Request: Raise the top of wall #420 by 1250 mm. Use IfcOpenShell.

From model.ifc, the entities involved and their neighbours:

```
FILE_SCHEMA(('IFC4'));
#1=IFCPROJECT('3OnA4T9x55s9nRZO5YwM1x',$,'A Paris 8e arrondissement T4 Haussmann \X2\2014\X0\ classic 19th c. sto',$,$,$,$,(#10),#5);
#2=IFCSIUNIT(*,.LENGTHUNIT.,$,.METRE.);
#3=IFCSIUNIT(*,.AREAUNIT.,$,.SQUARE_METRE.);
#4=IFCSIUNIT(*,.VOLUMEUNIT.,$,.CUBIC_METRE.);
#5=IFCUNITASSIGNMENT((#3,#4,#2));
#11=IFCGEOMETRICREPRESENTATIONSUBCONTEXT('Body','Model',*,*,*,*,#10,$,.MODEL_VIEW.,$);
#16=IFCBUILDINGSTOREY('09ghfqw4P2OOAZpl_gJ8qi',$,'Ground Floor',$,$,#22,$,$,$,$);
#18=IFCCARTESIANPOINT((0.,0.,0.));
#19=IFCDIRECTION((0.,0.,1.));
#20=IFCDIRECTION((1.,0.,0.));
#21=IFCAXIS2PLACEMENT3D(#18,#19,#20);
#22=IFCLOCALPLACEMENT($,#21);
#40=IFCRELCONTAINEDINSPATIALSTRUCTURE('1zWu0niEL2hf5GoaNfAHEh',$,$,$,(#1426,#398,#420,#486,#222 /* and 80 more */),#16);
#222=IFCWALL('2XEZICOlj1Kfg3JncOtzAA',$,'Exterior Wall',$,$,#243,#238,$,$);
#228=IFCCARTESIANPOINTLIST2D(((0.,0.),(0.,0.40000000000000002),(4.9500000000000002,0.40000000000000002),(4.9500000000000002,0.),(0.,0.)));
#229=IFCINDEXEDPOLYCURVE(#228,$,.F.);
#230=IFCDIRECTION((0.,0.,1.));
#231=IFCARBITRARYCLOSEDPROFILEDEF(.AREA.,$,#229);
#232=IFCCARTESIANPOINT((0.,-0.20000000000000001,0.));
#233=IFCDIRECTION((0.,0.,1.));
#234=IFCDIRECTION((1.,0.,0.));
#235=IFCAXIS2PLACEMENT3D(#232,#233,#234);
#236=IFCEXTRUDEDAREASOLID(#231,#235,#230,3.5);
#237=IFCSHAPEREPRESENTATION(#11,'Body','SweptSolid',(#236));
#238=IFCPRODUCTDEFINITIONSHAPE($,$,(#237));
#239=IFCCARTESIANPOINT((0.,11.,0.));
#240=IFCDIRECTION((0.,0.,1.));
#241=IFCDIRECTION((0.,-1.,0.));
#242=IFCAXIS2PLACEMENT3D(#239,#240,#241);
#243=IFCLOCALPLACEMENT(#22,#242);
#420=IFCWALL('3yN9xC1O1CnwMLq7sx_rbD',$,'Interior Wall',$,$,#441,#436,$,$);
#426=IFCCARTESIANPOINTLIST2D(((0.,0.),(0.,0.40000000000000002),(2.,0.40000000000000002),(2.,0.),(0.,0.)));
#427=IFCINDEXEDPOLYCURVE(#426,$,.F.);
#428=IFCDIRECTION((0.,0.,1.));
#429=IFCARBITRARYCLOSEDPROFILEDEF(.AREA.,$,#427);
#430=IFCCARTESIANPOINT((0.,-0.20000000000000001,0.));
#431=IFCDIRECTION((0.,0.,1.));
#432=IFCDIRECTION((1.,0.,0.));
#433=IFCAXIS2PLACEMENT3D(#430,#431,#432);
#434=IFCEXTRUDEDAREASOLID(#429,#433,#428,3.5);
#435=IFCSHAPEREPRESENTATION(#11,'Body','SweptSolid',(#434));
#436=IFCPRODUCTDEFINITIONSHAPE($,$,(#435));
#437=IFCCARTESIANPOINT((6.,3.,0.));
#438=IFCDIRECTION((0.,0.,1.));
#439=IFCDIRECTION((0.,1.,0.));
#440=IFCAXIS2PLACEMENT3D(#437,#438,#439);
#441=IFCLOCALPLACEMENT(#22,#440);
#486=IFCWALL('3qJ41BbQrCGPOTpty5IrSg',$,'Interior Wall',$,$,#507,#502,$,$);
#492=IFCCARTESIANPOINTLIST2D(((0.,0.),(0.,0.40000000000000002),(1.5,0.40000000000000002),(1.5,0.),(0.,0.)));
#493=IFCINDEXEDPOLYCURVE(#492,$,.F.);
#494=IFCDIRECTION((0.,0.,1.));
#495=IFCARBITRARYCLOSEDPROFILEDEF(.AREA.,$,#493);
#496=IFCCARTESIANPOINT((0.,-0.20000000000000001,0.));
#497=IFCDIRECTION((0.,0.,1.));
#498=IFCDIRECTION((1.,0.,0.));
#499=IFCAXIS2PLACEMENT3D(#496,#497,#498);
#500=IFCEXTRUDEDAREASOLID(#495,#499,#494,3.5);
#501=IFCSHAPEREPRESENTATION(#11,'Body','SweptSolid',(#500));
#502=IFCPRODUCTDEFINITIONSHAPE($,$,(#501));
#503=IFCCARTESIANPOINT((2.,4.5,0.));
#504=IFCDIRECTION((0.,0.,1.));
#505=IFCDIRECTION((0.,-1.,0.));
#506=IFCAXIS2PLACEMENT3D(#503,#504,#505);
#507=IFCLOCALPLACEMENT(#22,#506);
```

```python
import ifcopenshell
import ifcopenshell.geom
import ifcopenshell.util.representation
import ifcopenshell.util.shape

model = ifcopenshell.open("model.ifc")
settings = ifcopenshell.geom.settings()


def volume(element):
    """Net volume in cubic metres, openings subtracted."""
    shape = ifcopenshell.geom.create_shape(settings, element)
    return ifcopenshell.util.shape.get_volume(shape.geometry)


wall = model.by_id(420)
before = volume(wall)

body = ifcopenshell.util.representation.get_representation(wall, "Model", "Body")
solid = body.Items[0]
old_height = solid.Depth
solid.Depth += 1.25
after = volume(wall)

print(f"height {old_height:g} -> {solid.Depth:g}, volume {before:.3f} -> {after:.3f} m3")

model.write("model_rev.ifc")
```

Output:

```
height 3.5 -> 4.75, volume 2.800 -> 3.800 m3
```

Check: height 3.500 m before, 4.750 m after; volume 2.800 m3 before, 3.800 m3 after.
